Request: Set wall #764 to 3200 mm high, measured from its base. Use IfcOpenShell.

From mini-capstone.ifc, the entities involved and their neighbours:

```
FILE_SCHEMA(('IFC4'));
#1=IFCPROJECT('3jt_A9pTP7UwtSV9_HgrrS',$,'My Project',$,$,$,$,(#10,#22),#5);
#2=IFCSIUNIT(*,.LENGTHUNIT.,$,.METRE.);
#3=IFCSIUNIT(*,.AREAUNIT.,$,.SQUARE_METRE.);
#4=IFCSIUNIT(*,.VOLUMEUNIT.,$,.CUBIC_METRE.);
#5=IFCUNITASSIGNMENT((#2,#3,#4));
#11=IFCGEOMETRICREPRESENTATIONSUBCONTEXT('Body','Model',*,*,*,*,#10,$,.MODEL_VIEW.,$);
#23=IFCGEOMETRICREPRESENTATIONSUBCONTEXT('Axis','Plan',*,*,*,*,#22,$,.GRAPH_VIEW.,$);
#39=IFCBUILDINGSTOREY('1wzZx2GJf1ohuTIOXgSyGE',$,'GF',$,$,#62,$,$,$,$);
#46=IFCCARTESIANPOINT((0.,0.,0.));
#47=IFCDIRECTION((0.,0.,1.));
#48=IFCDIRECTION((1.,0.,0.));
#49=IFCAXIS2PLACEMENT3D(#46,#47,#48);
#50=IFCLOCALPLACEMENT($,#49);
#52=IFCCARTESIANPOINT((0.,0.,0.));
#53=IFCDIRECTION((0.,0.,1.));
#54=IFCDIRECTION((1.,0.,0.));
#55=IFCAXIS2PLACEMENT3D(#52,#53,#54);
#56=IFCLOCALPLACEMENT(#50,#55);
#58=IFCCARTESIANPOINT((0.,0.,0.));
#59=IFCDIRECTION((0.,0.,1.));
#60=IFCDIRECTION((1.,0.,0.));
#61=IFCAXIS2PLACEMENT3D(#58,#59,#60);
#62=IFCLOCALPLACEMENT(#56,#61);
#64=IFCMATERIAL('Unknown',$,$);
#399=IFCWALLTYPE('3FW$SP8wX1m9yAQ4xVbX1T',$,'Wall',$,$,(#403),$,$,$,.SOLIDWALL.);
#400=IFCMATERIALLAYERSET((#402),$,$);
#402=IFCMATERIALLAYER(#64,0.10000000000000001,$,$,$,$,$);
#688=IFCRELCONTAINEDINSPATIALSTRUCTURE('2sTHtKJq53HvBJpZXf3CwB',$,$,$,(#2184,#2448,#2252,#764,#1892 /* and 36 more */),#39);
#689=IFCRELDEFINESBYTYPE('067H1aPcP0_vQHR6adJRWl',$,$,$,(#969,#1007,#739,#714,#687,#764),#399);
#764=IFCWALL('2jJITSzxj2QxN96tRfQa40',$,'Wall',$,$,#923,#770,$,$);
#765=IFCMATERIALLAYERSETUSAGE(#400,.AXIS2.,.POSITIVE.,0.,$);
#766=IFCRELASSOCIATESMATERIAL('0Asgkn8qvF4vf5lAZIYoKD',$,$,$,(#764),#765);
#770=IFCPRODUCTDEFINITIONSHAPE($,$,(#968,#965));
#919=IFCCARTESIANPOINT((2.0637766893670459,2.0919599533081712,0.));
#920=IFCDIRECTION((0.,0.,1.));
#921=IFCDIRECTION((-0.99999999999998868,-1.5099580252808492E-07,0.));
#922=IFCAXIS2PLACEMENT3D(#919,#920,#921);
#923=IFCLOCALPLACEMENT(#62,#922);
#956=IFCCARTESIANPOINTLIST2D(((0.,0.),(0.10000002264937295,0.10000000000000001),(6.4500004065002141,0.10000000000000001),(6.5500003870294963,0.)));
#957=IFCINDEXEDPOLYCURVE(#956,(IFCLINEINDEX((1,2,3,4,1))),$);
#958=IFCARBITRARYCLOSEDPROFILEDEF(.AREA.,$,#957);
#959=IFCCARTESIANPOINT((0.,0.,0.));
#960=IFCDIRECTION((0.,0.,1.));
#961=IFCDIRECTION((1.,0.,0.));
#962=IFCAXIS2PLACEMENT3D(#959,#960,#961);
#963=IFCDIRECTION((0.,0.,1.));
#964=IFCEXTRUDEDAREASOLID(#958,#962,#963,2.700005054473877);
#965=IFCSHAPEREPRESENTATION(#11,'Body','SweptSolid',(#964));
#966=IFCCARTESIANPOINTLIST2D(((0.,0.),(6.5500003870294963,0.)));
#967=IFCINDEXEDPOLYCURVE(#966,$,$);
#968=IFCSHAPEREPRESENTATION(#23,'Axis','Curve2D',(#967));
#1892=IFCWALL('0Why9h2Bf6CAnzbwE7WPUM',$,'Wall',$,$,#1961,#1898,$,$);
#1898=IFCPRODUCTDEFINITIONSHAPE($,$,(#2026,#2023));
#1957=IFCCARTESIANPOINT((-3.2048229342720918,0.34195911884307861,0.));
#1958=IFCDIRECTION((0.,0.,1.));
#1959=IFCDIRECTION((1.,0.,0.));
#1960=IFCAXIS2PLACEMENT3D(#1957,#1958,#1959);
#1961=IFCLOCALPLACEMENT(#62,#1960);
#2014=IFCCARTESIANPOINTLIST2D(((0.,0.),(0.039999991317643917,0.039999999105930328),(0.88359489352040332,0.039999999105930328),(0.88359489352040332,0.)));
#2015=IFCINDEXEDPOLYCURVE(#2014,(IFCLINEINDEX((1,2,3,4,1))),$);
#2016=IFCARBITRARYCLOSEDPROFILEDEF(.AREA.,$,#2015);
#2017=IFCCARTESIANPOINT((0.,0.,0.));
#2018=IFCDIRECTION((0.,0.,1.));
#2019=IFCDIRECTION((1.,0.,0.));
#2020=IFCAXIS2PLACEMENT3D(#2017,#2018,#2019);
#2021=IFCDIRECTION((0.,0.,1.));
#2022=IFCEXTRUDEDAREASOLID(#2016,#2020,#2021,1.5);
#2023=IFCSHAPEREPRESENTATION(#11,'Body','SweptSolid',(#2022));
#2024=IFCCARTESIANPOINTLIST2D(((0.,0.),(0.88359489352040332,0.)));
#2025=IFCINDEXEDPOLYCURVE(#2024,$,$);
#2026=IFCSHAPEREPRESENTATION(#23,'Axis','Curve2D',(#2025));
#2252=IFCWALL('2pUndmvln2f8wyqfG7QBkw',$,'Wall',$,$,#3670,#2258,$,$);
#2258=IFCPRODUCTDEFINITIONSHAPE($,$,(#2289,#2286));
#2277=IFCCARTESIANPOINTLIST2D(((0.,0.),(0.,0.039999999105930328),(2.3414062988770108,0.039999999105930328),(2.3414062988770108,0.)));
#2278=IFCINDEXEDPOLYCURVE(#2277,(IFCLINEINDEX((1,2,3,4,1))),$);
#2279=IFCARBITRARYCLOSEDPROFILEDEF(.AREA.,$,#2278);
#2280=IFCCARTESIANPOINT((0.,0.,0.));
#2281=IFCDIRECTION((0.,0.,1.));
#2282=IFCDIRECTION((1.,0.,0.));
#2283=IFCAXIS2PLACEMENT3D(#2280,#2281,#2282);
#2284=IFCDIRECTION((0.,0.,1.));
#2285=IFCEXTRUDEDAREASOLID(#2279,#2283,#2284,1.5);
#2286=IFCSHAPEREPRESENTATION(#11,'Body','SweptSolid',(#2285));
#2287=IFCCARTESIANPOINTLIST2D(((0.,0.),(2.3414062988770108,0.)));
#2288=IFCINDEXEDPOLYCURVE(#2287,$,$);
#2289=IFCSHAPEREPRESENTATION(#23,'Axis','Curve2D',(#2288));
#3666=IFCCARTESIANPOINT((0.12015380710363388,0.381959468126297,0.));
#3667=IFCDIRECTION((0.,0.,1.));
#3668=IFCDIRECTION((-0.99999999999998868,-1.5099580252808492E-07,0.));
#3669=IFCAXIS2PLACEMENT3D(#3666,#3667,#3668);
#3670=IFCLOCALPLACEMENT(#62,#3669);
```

```python
import ifcopenshell
import ifcopenshell.geom
import ifcopenshell.util.representation
import ifcopenshell.util.shape

model = ifcopenshell.open("mini-capstone.ifc")
settings = ifcopenshell.geom.settings()


def volume(element):
    """Net volume in cubic metres, openings subtracted."""
    shape = ifcopenshell.geom.create_shape(settings, element)
    return ifcopenshell.util.shape.get_volume(shape.geometry)


wall = model.by_id(764)
before = volume(wall)

body = ifcopenshell.util.representation.get_representation(wall, "Model", "Body")
solid = body.Items[0]
old_height = solid.Depth
solid.Depth = 3.2
after = volume(wall)

print(f"height {old_height:g} -> {solid.Depth:g}, volume {before:.3f} -> {after:.3f} m3")

model.write("mini-capstone_updated.ifc")
```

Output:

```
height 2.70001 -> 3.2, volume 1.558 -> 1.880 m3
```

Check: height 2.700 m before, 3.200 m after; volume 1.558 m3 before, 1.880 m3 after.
